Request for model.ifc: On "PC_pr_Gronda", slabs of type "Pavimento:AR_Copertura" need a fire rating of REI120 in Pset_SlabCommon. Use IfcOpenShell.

First a look at what the model holds.

```python
import ifcopenshell
import ifcopenshell.util.element

model = ifcopenshell.open("model.ifc")
print(model.schema)
storey = next(s for s in model.by_type("IfcBuildingStorey") if s.Name == "PC_pr_Gronda")
slabs = [e for e in ifcopenshell.util.element.get_decomposition(storey) if e.is_a("IfcSlab")]
seen = {}
for e in slabs:
    element_type = ifcopenshell.util.element.get_type(e)
    key = (element_type.Name if element_type != e and element_type else None, ifcopenshell.util.element.get_pset(e, "Pset_SlabCommon", "FireRating"))
    seen[key] = seen.get(key, 0) + 1
for (name, value), count in sorted(seen.items(), key=str):
    print(count, "x", name, "|", value)
```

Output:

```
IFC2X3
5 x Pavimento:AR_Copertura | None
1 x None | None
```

```python
import ifcopenshell
import ifcopenshell.api.pset
import ifcopenshell.util.element

model = ifcopenshell.open("model.ifc")

storey = next(s for s in model.by_type("IfcBuildingStorey") if s.Name == "PC_pr_Gronda")
slabs = [e for e in ifcopenshell.util.element.get_decomposition(storey) if e.is_a("IfcSlab")]

count = 0
for e in slabs:
    element_type = ifcopenshell.util.element.get_type(e)
    if element_type in (None, e) or element_type.Name != "Pavimento:AR_Copertura":
        continue
    # add_pset returns the element's existing set when there is one.
    pset = ifcopenshell.api.pset.add_pset(model, product=e, name="Pset_SlabCommon")
    ifcopenshell.api.pset.edit_pset(model, pset=pset, properties={"FireRating": "REI120"})
    count += 1

print(count, "slabs updated")

model.write("model_updated.ifc")
```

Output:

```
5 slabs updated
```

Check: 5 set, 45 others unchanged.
